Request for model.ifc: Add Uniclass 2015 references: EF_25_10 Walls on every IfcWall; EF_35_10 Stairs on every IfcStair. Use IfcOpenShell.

First a look at what the model holds.

```python
import ifcopenshell

model = ifcopenshell.open("model.ifc")
print(model.schema)
print("classifications:", [c.Name for c in model.by_type("IfcClassification")])
for ifc_class in ("IfcDoor", "IfcRoof", "IfcStair", "IfcWall", "IfcWindow"):
    print(ifc_class, len(model.by_type(ifc_class)))
```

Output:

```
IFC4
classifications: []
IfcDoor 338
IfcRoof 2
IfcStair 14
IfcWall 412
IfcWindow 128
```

```python
import ifcopenshell
import ifcopenshell.api.classification

model = ifcopenshell.open("model.ifc")

system = ifcopenshell.api.classification.add_classification(model, classification="Uniclass 2015")

codes = {
    "IfcWall": ("EF_25_10", "Walls"),
    "IfcStair": ("EF_35_10", "Stairs"),
}
for ifc_class, (code, name) in codes.items():
    products = model.by_type(ifc_class)
    ifcopenshell.api.classification.add_reference(
        model, products=products, classification=system, identification=code, name=name
    )
    print(code, len(products))

model.write("model-out.ifc")
```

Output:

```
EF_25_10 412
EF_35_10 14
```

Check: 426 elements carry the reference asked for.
